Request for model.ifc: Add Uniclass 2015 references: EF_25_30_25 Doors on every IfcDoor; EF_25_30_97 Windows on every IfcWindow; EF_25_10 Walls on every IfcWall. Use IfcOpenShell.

First a look at what the model holds.

```python
import ifcopenshell

model = ifcopenshell.open("model.ifc")
print(model.schema)
print("classifications:", [c.Name for c in model.by_type("IfcClassification")])
for ifc_class in ("IfcDoor", "IfcRoof", "IfcStair", "IfcWall", "IfcWindow"):
    print(ifc_class, len(model.by_type(ifc_class)))
```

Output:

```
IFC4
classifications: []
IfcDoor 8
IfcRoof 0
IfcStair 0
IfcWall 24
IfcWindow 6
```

```python
import ifcopenshell
import ifcopenshell.api.classification

model = ifcopenshell.open("model.ifc")

system = ifcopenshell.api.classification.add_classification(model, classification="Uniclass 2015")

codes = {
    "IfcDoor": ("EF_25_30_25", "Doors"),
    "IfcWindow": ("EF_25_30_97", "Windows"),
    "IfcWall": ("EF_25_10", "Walls"),
}
for ifc_class, (code, name) in codes.items():
    products = model.by_type(ifc_class)
    ifcopenshell.api.classification.add_reference(
        model, products=products, classification=system, identification=code, name=name
    )
    print(code, len(products))

model.write("model-out.ifc")
```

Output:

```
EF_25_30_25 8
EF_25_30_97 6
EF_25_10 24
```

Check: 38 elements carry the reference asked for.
